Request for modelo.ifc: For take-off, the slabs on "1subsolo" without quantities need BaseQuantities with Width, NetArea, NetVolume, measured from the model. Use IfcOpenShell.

First a look at what the model holds.

```python
import ifcopenshell
import ifcopenshell.util.element
import ifcopenshell.util.unit

model = ifcopenshell.open("modelo.ifc")
print(model.schema)
for unit_type in ("LENGTHUNIT", "AREAUNIT", "VOLUMEUNIT"):
    print(unit_type, ifcopenshell.util.unit.calculate_unit_scale(model, unit_type))
storey = next(s for s in model.by_type("IfcBuildingStorey") if s.Name == "1subsolo")
slabs = [e for e in ifcopenshell.util.element.get_decomposition(storey) if e.is_a("IfcSlab")]
for e in sorted(slabs, key=lambda e: e.id()):
    print(e.id(), e.is_a(), e.Name, list(ifcopenshell.util.element.get_psets(e, qtos_only=True)), sep=" | ")
```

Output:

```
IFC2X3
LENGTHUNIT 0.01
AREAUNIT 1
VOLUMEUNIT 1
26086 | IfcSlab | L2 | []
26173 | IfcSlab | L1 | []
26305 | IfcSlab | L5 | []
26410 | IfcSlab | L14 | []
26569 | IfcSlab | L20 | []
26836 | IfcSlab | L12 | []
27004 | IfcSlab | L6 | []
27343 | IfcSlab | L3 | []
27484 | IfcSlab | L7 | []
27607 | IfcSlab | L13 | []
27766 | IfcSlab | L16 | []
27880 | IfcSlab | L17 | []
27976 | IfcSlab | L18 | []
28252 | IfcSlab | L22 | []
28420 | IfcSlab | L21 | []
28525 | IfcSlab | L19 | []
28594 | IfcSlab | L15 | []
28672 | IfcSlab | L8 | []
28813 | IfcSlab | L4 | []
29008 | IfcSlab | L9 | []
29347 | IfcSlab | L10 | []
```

```python
import ifcopenshell
import ifcopenshell.api.pset
import ifcopenshell.geom
import ifcopenshell.util.element
import ifcopenshell.util.shape
import ifcopenshell.util.unit

model = ifcopenshell.open("modelo.ifc")
unit_scale = ifcopenshell.util.unit.calculate_unit_scale(model)
area_scale = ifcopenshell.util.unit.calculate_unit_scale(model, "AREAUNIT")
volume_scale = ifcopenshell.util.unit.calculate_unit_scale(model, "VOLUMEUNIT")
settings = ifcopenshell.geom.settings()

storey = next(s for s in model.by_type("IfcBuildingStorey") if s.Name == "1subsolo")
slabs = [e for e in ifcopenshell.util.element.get_decomposition(storey) if e.is_a("IfcSlab")]

for e in sorted(slabs, key=lambda e: e.id()):
    if ifcopenshell.util.element.get_psets(e, qtos_only=True, should_inherit=False):
        continue
    # Geometry comes back in metres, in the element's own axes.
    shape = ifcopenshell.geom.create_shape(settings, e)
    values = {
        "Width": ifcopenshell.util.shape.get_z(shape.geometry) / unit_scale,
        "NetArea": ifcopenshell.util.shape.get_footprint_area(shape.geometry) / area_scale,
        "NetVolume": ifcopenshell.util.shape.get_volume(shape.geometry) / volume_scale,
    }
    qto = ifcopenshell.api.pset.add_qto(model, product=e, name="BaseQuantities")
    ifcopenshell.api.pset.edit_qto(model, qto=qto, properties=values)
    print(e.id(), {k: round(v, 3) for k, v in values.items()})

model.write("modelo-out.ifc")
```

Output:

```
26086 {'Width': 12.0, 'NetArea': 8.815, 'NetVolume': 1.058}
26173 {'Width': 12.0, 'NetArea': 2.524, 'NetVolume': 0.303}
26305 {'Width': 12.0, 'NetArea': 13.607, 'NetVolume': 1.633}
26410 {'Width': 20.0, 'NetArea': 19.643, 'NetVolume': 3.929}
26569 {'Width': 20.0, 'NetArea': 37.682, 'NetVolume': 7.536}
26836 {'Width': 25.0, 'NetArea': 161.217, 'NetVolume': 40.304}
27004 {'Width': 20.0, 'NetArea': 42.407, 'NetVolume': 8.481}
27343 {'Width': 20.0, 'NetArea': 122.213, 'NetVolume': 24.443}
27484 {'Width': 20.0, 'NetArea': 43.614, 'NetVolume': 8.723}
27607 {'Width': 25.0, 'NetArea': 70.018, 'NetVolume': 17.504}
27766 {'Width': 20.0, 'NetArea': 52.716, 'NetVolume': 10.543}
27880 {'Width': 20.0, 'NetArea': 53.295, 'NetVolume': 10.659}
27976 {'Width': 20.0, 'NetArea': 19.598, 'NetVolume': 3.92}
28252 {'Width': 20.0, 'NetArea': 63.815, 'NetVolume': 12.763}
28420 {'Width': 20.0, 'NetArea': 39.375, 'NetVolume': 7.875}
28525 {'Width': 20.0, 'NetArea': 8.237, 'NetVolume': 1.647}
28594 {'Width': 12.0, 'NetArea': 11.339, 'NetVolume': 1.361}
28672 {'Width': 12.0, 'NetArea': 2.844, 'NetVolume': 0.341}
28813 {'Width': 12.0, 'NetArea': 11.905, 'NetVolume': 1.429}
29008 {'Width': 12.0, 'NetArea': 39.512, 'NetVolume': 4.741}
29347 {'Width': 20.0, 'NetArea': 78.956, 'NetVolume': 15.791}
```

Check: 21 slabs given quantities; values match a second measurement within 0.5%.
